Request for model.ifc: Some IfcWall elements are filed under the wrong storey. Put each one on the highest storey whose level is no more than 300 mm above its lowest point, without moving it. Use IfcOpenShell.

First a look at what the model holds.

```python
import ifcopenshell
import ifcopenshell.util.element
import ifcopenshell.util.placement

model = ifcopenshell.open("model.ifc")
print(model.schema)
for storey in model.by_type("IfcBuildingStorey"):
    level = ifcopenshell.util.placement.get_storey_elevation(storey)
    count = sum(e.is_a("IfcWall") for e in ifcopenshell.util.element.get_contained(storey))
    print(storey.id(), storey.Name, round(level, 3), count, sep=" | ")
```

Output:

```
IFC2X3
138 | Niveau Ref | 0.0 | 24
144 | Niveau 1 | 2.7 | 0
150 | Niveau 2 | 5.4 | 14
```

```python
import ifcopenshell
import ifcopenshell.api.spatial
import ifcopenshell.geom
import ifcopenshell.util.element
import ifcopenshell.util.placement
import ifcopenshell.util.shape
import ifcopenshell.util.unit

model = ifcopenshell.open("model.ifc")
unit_scale = ifcopenshell.util.unit.calculate_unit_scale(model)
settings = ifcopenshell.geom.settings()

levels = sorted(
    ((ifcopenshell.util.placement.get_storey_elevation(s) * unit_scale, s) for s in model.by_type("IfcBuildingStorey")),
    key=lambda pair: pair[0],
)

for e in model.by_type("IfcWall"):
    current = e.ContainedInStructure[0].RelatingStructure if e.ContainedInStructure else None
    if current is None or not current.is_a("IfcBuildingStorey"):
        continue
    shape = ifcopenshell.geom.create_shape(settings, e)
    bottom = ifcopenshell.util.shape.get_shape_bottom_elevation(shape, shape.geometry)
    below = [s for level, s in levels if level <= bottom + 0.3]
    storey = below[-1] if below else levels[0][1]
    if storey != current:
        # assign_container keeps the world position.
        ifcopenshell.api.spatial.assign_container(model, products=[e], relating_structure=storey)
        print(e.id(), current.Name, "->", storey.Name)

model.write("model_edited.ifc")
```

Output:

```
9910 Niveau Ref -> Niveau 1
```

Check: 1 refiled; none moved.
